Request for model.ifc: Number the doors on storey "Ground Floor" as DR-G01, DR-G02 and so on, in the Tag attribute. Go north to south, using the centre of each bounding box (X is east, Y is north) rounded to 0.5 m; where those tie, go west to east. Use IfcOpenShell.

First a look at what the model holds.

```python
import ifcopenshell
import ifcopenshell.util.element
import ifcopenshell.util.placement

model = ifcopenshell.open("model.ifc")
print(model.schema)
storey = next(s for s in model.by_type("IfcBuildingStorey") if s.Name == "Ground Floor")
doors = [e for e in ifcopenshell.util.element.get_decomposition(storey) if e.is_a("IfcDoor")]
for e in sorted(doors, key=lambda e: e.id()):
    origin = ifcopenshell.util.placement.get_local_placement(e.ObjectPlacement)[:3, 3]
    print(e.id(), e.Tag, e.Name, origin.round(2) + 0.0, sep=" | ")
```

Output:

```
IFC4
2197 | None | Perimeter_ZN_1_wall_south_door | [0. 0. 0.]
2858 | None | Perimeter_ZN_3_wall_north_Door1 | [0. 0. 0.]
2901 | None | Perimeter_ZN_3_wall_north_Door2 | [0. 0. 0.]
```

```python
import ifcopenshell
import ifcopenshell.geom
import ifcopenshell.util.element
import ifcopenshell.util.shape

model = ifcopenshell.open("model.ifc")
settings = ifcopenshell.geom.settings()
settings.set("use-world-coords", True)


def centre(element):
    shape = ifcopenshell.geom.create_shape(settings, element)
    return ifcopenshell.util.shape.get_bbox_centroid(shape.geometry)


storey = next(s for s in model.by_type("IfcBuildingStorey") if s.Name == "Ground Floor")
doors = [e for e in ifcopenshell.util.element.get_decomposition(storey) if e.is_a("IfcDoor")]

# Insertion points can sit at a corner or the storey origin, so sort by the geometry (in metres).
centres = {e: centre(e) for e in doors}
doors.sort(key=lambda e: (-round(centres[e][1] / 0.5), centres[e][0]))

for i, e in enumerate(doors, start=1):
    number = f"DR-G{i:02d}"
    e.Tag = number
    print(e.id(), number)

model.write("model_edited.ifc")
```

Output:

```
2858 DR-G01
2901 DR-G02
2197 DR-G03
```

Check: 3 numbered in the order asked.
